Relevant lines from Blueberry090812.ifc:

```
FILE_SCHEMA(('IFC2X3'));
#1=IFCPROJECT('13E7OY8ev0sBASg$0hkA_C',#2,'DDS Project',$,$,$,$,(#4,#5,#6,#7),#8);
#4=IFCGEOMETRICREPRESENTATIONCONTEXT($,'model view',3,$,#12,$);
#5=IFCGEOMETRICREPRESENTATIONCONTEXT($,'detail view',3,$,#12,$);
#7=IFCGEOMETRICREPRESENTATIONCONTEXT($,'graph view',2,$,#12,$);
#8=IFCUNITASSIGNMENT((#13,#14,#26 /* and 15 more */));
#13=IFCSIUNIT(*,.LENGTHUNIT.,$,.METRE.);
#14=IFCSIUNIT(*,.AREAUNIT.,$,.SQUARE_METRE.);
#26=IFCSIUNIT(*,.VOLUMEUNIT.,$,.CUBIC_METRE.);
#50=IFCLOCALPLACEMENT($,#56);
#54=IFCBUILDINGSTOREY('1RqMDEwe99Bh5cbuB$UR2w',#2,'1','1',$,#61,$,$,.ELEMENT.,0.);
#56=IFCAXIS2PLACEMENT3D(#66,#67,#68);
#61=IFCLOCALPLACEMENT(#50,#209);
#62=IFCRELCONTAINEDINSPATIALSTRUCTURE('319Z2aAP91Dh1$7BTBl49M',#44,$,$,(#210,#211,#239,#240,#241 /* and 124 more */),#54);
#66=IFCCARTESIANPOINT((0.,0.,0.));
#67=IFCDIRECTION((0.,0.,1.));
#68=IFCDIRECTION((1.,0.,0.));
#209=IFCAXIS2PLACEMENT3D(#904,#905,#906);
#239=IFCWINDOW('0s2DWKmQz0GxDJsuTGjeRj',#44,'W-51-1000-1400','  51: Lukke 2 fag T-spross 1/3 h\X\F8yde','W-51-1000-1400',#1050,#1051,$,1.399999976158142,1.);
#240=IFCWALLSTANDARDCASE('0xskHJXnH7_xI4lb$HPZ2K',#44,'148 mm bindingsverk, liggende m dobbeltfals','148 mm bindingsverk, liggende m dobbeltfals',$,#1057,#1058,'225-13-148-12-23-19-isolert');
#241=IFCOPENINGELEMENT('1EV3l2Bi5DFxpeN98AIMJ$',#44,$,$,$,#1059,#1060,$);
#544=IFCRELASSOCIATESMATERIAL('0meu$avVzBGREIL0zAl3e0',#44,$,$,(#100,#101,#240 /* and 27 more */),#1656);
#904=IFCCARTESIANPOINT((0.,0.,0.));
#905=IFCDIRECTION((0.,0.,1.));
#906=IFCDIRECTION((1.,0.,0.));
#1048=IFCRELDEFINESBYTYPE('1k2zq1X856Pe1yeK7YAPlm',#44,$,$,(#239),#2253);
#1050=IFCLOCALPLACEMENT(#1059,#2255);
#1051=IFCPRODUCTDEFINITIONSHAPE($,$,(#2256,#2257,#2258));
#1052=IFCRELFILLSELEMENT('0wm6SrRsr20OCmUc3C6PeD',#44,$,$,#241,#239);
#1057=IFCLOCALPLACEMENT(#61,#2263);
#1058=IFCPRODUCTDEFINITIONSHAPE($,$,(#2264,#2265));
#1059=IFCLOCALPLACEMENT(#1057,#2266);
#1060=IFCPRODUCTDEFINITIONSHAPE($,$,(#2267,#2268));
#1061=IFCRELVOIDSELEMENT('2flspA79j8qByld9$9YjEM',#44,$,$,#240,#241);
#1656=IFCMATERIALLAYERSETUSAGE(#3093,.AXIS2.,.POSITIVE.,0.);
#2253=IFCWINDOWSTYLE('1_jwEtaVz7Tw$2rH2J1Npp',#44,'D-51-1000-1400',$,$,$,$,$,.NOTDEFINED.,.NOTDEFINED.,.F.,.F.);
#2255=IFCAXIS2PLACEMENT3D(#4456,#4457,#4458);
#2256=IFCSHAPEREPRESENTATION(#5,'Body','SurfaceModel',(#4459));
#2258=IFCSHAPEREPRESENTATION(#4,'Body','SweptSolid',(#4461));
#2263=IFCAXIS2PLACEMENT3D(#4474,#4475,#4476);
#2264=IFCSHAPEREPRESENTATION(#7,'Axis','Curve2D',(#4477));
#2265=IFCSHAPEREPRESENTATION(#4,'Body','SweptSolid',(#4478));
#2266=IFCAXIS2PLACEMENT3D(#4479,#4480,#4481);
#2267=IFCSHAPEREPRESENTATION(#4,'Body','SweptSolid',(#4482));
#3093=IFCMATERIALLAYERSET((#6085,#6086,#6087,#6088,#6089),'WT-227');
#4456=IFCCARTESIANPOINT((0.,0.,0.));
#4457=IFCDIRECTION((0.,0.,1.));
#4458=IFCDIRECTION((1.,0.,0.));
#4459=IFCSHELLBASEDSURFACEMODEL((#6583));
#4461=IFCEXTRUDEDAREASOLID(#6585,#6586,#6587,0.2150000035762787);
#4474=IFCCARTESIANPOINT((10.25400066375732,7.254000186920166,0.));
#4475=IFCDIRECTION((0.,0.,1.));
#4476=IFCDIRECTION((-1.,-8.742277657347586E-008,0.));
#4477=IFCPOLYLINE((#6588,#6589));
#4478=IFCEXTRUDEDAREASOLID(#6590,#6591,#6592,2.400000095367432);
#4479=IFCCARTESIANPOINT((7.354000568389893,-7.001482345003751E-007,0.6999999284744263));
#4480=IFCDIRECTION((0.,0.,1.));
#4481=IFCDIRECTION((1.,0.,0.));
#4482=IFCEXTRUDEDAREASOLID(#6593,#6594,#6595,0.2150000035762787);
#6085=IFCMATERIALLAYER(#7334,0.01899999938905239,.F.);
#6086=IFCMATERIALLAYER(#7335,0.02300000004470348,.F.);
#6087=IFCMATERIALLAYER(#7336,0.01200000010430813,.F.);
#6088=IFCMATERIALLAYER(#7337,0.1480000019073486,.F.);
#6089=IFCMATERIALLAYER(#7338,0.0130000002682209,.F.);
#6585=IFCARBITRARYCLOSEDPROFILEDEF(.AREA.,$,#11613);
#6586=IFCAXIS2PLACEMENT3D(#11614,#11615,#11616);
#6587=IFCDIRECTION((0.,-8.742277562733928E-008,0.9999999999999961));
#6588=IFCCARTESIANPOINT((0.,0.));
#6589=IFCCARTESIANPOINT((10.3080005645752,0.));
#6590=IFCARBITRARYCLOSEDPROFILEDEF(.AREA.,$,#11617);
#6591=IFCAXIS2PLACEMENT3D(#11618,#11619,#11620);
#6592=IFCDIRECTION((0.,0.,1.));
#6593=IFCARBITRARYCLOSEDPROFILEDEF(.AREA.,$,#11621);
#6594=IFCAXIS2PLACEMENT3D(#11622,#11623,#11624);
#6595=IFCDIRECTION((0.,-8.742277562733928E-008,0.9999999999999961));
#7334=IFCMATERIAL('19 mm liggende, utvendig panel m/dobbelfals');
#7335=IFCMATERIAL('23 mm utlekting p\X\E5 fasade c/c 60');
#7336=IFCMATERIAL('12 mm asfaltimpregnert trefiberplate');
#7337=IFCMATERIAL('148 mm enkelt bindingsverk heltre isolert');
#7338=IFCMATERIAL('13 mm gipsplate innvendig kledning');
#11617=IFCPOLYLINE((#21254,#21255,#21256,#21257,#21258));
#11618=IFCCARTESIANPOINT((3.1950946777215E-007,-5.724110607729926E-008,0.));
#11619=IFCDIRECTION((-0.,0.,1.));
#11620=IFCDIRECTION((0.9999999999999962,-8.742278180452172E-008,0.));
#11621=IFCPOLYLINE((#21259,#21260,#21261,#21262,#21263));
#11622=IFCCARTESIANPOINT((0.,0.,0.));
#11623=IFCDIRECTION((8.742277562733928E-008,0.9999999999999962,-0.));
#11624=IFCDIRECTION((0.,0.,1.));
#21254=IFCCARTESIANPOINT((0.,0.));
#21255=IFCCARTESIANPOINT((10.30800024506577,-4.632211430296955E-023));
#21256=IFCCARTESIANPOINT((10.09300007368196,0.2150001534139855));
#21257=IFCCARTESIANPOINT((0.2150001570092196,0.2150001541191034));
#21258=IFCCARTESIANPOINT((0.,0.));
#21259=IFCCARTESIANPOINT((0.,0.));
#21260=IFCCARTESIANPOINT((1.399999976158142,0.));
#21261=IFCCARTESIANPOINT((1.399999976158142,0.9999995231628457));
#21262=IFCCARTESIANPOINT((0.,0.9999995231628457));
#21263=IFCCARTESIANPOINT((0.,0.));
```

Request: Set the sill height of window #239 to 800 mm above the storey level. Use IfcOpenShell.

```python
import numpy as np
import ifcopenshell
import ifcopenshell.api.geometry
import ifcopenshell.geom
import ifcopenshell.util.element
import ifcopenshell.util.placement
import ifcopenshell.util.shape
import ifcopenshell.util.unit

model = ifcopenshell.open("Blueberry090812.ifc")
unit_scale = ifcopenshell.util.unit.calculate_unit_scale(model)

window = model.by_guid("0s2DWKmQz0GxDJsuTGjeRj")
opening = window.FillsVoids[0].RelatingOpeningElement
storey = ifcopenshell.util.element.get_container(window, ifc_class="IfcBuildingStorey")
level = ifcopenshell.util.placement.get_local_placement(storey.ObjectPlacement)[2, 3]

# The opening's origin need not be at the sill, so measure its lowest point.
shape = ifcopenshell.geom.create_shape(ifcopenshell.geom.settings(), opening)
bottom = ifcopenshell.util.shape.get_shape_bottom_elevation(shape, shape.geometry) / unit_scale
dz = level + 0.8 / unit_scale - bottom

shift = np.array([0.0, 0.0, dz])
# The window is placed relative to its opening, so it follows when the opening moves.
matrix = ifcopenshell.util.placement.get_local_placement(opening.ObjectPlacement)
matrix[:3, 3] += shift
ifcopenshell.api.geometry.edit_object_placement(
    model, product=opening, matrix=matrix, is_si=False, should_transform_children=True
)

print(f"moved by {dz * unit_scale:+.3f} m")

model.write("Blueberry090812_v2.ifc")
```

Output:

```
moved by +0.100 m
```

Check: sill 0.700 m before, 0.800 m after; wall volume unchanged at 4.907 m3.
